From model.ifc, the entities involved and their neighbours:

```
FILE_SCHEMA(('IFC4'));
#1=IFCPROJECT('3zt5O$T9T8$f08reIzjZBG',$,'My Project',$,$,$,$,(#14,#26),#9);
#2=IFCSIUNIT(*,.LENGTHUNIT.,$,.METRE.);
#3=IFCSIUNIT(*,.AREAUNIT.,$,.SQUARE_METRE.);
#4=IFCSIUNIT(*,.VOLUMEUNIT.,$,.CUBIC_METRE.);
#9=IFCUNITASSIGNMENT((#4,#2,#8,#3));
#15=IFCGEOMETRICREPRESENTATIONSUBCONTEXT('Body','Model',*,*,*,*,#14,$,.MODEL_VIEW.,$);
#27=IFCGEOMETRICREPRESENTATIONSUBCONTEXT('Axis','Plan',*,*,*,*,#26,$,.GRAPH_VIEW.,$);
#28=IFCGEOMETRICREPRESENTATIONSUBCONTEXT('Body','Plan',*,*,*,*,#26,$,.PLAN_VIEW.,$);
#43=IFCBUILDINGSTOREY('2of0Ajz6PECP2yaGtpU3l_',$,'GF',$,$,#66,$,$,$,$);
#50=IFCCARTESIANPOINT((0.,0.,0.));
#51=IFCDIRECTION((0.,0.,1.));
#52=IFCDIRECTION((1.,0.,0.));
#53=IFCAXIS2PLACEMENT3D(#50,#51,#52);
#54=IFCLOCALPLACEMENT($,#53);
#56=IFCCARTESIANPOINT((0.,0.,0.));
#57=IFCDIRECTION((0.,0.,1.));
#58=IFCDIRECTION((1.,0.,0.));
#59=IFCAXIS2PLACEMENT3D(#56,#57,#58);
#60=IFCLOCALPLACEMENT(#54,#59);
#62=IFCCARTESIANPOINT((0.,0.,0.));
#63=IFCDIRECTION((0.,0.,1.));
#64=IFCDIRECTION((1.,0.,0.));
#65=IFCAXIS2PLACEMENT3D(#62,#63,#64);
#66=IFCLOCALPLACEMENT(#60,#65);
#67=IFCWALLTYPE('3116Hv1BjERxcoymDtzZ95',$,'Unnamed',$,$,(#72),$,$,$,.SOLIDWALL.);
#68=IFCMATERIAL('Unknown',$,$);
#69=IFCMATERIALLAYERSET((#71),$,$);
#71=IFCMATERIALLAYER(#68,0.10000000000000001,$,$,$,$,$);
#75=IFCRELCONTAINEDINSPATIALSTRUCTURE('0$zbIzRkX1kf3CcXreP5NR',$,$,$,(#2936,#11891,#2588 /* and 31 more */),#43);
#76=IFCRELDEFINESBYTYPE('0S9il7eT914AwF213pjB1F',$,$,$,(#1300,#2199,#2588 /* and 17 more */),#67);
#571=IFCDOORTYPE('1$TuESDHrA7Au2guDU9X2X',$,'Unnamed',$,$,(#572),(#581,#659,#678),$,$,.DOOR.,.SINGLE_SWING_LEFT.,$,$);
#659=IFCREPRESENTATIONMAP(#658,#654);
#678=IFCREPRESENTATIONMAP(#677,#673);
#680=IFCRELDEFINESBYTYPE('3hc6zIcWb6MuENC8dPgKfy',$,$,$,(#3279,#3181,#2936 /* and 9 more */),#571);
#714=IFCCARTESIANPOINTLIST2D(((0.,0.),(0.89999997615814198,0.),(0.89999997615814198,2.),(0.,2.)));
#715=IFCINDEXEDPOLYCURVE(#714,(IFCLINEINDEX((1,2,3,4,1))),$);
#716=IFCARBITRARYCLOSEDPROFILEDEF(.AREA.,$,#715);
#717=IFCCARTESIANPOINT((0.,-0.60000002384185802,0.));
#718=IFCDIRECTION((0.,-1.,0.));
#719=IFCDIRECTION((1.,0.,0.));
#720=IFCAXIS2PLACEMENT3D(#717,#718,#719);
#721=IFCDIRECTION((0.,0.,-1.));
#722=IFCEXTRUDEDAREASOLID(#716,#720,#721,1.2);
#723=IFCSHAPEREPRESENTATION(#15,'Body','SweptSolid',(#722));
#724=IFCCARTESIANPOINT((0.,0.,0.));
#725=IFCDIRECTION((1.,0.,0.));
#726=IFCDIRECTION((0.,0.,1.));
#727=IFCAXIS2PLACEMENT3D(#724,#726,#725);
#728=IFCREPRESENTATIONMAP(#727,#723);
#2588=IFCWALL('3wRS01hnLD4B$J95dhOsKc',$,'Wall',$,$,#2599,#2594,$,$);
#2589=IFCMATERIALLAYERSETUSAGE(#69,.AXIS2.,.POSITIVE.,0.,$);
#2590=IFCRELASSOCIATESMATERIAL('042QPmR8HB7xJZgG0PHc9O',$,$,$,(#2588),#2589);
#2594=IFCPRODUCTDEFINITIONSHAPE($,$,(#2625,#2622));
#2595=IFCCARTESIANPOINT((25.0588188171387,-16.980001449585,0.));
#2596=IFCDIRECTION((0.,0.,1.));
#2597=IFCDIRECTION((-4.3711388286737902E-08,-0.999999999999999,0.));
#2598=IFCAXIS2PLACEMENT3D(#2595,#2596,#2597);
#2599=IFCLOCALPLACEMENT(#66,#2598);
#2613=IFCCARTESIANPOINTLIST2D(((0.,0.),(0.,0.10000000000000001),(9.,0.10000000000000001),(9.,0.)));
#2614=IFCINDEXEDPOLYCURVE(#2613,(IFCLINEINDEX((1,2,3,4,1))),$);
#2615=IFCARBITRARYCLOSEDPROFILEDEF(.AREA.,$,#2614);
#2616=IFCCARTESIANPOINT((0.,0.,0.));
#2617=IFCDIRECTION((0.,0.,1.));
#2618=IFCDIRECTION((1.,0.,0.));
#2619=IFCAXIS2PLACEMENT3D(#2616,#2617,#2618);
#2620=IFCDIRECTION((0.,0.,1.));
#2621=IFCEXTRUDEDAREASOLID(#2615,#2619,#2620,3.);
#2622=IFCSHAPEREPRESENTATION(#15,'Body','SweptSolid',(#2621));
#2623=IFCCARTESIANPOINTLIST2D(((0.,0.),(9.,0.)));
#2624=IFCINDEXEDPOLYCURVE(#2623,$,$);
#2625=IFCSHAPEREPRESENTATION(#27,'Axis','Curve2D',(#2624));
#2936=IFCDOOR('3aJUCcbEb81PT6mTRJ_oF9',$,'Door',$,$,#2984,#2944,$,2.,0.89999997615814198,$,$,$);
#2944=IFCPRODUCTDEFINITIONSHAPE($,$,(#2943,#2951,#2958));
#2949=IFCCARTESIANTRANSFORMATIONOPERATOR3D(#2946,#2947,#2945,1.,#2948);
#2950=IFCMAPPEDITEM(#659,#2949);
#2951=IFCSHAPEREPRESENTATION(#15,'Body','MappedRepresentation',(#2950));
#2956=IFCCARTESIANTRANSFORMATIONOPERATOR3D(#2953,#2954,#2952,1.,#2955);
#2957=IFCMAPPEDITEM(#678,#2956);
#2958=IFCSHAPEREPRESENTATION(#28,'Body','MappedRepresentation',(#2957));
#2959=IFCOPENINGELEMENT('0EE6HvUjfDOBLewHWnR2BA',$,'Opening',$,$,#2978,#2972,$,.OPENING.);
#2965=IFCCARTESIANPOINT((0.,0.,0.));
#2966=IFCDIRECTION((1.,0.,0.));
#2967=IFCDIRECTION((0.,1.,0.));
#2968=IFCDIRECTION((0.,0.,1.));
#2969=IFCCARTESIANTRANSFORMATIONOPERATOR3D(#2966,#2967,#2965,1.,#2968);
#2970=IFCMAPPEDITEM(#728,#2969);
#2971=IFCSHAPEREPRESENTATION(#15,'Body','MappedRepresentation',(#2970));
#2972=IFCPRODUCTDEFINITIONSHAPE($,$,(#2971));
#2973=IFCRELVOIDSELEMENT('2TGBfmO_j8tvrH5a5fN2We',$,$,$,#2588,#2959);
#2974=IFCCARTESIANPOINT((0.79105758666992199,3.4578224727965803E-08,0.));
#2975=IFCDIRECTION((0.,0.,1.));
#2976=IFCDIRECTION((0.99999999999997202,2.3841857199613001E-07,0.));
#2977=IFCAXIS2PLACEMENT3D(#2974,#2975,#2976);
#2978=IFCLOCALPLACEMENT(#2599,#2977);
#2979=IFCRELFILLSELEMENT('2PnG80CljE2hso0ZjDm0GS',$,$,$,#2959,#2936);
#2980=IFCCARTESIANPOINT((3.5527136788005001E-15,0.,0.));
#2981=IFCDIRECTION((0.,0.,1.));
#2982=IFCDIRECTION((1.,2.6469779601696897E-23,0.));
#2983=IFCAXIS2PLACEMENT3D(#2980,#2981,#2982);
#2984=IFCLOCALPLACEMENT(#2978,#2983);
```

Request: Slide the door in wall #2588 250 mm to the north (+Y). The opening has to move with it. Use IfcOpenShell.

```python
import ifcopenshell
import ifcopenshell.api.geometry
import ifcopenshell.util.placement
import ifcopenshell.util.unit

model = ifcopenshell.open("model.ifc")
unit_scale = ifcopenshell.util.unit.calculate_unit_scale(model)

door = model.by_id(2936)
opening = door.FillsVoids[0].RelatingOpeningElement
wall = opening.VoidsElements[0].RelatingBuildingElement

wall_matrix = ifcopenshell.util.placement.get_local_placement(wall.ObjectPlacement)
shift = wall_matrix[:3, 0] * -0.25 / unit_scale
before = ifcopenshell.util.placement.get_local_placement(door.ObjectPlacement)[:3, 3].copy()

# The door is placed relative to its opening, so it follows when the opening moves.
matrix = ifcopenshell.util.placement.get_local_placement(opening.ObjectPlacement)
matrix[:3, 3] += shift
ifcopenshell.api.geometry.edit_object_placement(
    model, product=opening, matrix=matrix, is_si=False, should_transform_children=True
)

after = ifcopenshell.util.placement.get_local_placement(door.ObjectPlacement)[:3, 3]
print("door moved by", (after - before).round(3) + 0.0)

model.write("model-out.ifc")
```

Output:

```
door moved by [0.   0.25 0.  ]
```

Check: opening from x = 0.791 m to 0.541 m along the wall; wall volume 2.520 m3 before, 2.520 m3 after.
